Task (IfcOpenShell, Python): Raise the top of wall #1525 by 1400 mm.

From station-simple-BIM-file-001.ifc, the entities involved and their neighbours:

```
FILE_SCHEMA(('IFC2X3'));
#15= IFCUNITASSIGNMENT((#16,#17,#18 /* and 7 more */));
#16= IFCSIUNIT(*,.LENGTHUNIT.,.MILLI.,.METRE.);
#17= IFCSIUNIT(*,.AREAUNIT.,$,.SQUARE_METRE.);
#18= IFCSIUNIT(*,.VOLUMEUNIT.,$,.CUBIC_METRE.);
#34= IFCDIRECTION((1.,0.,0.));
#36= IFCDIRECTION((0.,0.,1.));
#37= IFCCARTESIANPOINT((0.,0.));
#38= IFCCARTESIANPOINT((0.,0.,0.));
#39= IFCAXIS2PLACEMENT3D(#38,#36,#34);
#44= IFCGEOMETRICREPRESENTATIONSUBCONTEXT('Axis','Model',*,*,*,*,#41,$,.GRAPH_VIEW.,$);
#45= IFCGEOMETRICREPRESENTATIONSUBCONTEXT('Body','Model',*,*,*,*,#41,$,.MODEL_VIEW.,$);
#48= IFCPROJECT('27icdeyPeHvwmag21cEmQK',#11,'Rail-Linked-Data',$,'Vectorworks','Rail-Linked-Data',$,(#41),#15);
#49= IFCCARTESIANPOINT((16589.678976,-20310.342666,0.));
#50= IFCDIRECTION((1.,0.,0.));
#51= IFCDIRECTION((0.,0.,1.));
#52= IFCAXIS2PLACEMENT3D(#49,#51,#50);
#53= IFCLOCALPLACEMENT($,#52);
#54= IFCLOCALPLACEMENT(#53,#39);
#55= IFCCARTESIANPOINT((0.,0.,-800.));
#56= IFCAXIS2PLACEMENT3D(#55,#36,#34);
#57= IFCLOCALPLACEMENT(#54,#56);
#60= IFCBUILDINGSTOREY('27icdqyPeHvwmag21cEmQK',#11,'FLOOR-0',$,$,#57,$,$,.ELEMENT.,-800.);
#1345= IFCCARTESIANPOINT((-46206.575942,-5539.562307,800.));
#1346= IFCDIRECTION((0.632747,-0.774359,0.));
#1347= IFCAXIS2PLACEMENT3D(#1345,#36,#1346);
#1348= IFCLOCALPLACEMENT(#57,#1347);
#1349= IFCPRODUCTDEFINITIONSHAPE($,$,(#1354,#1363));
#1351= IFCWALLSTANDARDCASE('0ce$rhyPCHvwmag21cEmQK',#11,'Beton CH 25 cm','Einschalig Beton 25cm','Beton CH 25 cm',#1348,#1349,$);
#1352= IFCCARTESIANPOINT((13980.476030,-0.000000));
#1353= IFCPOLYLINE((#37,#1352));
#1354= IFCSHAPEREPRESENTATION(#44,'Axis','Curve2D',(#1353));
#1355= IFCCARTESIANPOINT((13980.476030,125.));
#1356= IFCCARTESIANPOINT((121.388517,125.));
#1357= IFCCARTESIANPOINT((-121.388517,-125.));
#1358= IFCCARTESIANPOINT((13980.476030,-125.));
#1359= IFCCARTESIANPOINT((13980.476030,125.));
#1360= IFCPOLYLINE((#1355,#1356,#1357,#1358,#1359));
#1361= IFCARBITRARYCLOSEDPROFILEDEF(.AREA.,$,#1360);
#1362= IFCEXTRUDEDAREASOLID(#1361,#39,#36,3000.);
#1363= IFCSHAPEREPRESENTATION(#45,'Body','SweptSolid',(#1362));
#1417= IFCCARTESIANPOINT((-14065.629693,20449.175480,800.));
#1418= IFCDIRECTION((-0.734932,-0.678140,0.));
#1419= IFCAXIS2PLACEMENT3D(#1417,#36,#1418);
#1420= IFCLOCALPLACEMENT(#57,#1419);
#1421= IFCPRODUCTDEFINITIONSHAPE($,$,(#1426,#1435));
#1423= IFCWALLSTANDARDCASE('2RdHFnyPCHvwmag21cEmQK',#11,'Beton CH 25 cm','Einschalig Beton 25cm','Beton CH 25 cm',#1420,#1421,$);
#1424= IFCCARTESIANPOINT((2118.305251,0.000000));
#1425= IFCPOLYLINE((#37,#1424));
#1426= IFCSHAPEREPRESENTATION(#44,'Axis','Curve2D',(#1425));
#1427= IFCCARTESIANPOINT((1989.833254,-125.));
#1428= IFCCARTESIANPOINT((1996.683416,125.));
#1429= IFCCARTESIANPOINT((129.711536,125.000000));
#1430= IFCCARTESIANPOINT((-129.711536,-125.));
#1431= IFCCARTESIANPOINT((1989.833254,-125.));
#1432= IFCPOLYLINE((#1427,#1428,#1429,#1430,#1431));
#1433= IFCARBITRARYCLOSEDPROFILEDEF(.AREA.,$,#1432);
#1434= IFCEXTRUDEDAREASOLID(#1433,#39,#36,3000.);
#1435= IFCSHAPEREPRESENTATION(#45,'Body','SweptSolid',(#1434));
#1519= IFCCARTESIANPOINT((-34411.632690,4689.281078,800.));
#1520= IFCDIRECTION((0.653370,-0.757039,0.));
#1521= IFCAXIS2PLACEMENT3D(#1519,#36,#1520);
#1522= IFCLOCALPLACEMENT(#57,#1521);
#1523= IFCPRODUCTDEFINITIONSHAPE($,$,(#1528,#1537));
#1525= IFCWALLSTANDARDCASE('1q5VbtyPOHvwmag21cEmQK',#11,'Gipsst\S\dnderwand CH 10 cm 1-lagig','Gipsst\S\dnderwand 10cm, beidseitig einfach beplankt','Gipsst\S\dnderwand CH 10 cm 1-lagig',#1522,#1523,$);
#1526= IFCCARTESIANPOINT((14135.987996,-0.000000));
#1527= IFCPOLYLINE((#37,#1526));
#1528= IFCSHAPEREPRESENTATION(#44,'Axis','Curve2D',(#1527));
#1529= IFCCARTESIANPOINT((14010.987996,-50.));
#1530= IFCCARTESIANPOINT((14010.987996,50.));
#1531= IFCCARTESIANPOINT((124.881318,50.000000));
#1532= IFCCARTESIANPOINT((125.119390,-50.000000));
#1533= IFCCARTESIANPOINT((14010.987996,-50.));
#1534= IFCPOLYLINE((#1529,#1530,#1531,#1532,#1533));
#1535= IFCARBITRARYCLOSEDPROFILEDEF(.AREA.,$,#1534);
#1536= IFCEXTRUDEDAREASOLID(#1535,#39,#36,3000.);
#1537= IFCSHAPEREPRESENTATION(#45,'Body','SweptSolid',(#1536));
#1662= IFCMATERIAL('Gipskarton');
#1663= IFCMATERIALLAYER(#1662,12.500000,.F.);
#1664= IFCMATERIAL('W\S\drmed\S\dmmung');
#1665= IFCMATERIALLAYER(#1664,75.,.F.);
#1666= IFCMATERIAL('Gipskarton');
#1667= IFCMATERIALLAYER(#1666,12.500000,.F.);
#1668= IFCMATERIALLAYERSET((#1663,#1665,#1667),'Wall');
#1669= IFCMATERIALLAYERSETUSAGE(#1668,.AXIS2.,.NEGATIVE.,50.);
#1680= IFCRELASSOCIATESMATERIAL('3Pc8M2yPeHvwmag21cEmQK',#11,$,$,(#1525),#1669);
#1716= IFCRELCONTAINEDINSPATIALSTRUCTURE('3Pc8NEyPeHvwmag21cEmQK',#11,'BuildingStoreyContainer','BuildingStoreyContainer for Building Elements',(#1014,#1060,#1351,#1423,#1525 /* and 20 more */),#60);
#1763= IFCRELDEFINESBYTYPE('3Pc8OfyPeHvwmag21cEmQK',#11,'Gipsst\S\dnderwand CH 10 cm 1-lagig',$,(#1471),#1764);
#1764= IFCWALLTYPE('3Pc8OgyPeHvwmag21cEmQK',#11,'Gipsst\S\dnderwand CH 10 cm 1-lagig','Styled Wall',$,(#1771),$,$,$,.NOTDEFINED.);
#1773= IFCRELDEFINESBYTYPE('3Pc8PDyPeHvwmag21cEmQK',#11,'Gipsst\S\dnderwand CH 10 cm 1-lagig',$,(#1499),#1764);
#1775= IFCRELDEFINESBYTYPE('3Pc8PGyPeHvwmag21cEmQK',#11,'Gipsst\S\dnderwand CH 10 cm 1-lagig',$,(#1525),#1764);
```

```python
import ifcopenshell
import ifcopenshell.geom
import ifcopenshell.util.representation
import ifcopenshell.util.shape
import ifcopenshell.util.unit

model = ifcopenshell.open("station-simple-BIM-file-001.ifc")
unit_scale = ifcopenshell.util.unit.calculate_unit_scale(model)
settings = ifcopenshell.geom.settings()


def volume(element):
    """Net volume in cubic metres, openings subtracted."""
    shape = ifcopenshell.geom.create_shape(settings, element)
    return ifcopenshell.util.shape.get_volume(shape.geometry)


wall = model.by_guid("1q5VbtyPOHvwmag21cEmQK")
before = volume(wall)

body = ifcopenshell.util.representation.get_representation(wall, "Model", "Body")
solid = body.Items[0]
old_height = solid.Depth
solid.Depth += 1.4 / unit_scale
after = volume(wall)

print(f"height {old_height:g} -> {solid.Depth:g}, volume {before:.3f} -> {after:.3f} m3")

model.write("station-simple-BIM-file-001_edited.ifc")
```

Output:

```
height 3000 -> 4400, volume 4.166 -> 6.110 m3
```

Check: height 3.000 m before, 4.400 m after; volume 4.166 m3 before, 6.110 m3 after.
